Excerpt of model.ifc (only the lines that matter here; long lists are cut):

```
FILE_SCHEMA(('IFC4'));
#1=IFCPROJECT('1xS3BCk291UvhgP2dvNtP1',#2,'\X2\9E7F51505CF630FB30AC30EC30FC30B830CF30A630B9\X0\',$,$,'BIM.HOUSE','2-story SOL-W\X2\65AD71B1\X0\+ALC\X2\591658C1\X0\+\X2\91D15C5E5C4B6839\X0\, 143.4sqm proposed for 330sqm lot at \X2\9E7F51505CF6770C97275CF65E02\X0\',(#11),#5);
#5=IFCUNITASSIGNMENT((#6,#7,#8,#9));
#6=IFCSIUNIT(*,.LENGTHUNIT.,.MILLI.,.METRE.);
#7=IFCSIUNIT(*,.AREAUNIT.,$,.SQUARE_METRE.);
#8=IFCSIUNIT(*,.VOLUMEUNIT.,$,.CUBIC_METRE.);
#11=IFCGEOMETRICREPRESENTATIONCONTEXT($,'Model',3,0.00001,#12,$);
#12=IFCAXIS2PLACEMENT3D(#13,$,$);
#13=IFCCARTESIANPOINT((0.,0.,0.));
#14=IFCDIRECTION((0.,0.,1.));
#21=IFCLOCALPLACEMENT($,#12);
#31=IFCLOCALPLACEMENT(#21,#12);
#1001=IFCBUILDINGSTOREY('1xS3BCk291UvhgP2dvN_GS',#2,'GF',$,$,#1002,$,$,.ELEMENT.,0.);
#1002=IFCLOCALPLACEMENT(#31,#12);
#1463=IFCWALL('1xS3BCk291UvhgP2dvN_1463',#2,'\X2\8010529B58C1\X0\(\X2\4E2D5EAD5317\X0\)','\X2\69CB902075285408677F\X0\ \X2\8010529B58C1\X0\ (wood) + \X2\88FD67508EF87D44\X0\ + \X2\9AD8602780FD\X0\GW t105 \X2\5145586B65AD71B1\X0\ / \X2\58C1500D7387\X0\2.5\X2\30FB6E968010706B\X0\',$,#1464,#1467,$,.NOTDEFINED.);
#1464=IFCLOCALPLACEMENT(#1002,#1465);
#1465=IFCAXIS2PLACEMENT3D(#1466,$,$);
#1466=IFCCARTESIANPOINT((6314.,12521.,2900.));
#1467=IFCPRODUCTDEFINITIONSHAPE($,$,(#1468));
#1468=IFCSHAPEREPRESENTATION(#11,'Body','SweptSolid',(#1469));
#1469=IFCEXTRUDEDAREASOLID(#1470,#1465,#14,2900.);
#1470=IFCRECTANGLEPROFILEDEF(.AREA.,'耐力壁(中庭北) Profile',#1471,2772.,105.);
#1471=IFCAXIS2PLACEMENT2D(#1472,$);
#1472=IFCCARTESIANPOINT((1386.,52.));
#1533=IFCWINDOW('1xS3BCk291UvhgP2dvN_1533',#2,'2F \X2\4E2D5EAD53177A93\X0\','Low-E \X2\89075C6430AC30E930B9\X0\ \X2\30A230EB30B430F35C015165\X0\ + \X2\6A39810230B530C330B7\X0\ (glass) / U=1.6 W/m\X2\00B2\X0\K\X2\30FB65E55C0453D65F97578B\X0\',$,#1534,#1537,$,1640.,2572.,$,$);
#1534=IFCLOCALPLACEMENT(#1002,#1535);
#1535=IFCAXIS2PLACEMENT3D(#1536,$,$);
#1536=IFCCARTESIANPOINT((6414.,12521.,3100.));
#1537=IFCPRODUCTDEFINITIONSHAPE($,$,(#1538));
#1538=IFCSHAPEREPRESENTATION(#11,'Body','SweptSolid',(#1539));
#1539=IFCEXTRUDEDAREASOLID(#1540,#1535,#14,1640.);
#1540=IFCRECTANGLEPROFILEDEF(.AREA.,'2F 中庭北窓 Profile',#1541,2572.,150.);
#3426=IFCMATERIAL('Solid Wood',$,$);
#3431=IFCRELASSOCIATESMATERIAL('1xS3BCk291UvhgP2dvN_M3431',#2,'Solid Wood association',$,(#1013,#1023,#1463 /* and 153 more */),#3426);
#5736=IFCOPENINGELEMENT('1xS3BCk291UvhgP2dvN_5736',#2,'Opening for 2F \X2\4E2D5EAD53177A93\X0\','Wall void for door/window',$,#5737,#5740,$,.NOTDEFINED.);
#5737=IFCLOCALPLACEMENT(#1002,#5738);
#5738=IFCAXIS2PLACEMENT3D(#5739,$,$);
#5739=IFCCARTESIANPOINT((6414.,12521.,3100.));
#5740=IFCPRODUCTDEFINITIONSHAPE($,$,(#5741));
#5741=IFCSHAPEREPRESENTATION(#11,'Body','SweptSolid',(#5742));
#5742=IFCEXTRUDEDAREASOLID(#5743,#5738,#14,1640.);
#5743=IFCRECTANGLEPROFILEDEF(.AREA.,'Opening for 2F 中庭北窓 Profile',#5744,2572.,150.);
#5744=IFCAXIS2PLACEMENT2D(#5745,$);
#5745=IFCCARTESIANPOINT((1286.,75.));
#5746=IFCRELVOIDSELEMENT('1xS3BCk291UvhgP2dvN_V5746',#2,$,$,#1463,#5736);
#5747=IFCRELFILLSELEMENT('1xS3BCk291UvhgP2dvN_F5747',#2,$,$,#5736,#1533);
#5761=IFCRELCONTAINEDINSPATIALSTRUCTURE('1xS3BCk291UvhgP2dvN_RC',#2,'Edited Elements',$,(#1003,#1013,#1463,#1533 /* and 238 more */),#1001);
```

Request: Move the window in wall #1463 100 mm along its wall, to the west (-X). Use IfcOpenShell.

```python
import ifcopenshell
import ifcopenshell.api.geometry
import ifcopenshell.util.placement

model = ifcopenshell.open("model.ifc")

window = model.by_id(1533)
opening = window.FillsVoids[0].RelatingOpeningElement
wall = opening.VoidsElements[0].RelatingBuildingElement

wall_matrix = ifcopenshell.util.placement.get_local_placement(wall.ObjectPlacement)
shift = wall_matrix[:3, 0] * -100.0
before = ifcopenshell.util.placement.get_local_placement(window.ObjectPlacement)[:3, 3].copy()

# The window is not placed relative to its opening, so move both.
for product in (opening, window):
    matrix = ifcopenshell.util.placement.get_local_placement(product.ObjectPlacement)
    matrix[:3, 3] += shift
    ifcopenshell.api.geometry.edit_object_placement(model, product=product, matrix=matrix, is_si=False)

after = ifcopenshell.util.placement.get_local_placement(window.ObjectPlacement)[:3, 3]
print("window moved by", (after - before).round(3) + 0.0)

model.write("model-out.ifc")
```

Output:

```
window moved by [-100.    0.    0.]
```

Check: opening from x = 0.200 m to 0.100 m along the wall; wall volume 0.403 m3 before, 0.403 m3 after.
